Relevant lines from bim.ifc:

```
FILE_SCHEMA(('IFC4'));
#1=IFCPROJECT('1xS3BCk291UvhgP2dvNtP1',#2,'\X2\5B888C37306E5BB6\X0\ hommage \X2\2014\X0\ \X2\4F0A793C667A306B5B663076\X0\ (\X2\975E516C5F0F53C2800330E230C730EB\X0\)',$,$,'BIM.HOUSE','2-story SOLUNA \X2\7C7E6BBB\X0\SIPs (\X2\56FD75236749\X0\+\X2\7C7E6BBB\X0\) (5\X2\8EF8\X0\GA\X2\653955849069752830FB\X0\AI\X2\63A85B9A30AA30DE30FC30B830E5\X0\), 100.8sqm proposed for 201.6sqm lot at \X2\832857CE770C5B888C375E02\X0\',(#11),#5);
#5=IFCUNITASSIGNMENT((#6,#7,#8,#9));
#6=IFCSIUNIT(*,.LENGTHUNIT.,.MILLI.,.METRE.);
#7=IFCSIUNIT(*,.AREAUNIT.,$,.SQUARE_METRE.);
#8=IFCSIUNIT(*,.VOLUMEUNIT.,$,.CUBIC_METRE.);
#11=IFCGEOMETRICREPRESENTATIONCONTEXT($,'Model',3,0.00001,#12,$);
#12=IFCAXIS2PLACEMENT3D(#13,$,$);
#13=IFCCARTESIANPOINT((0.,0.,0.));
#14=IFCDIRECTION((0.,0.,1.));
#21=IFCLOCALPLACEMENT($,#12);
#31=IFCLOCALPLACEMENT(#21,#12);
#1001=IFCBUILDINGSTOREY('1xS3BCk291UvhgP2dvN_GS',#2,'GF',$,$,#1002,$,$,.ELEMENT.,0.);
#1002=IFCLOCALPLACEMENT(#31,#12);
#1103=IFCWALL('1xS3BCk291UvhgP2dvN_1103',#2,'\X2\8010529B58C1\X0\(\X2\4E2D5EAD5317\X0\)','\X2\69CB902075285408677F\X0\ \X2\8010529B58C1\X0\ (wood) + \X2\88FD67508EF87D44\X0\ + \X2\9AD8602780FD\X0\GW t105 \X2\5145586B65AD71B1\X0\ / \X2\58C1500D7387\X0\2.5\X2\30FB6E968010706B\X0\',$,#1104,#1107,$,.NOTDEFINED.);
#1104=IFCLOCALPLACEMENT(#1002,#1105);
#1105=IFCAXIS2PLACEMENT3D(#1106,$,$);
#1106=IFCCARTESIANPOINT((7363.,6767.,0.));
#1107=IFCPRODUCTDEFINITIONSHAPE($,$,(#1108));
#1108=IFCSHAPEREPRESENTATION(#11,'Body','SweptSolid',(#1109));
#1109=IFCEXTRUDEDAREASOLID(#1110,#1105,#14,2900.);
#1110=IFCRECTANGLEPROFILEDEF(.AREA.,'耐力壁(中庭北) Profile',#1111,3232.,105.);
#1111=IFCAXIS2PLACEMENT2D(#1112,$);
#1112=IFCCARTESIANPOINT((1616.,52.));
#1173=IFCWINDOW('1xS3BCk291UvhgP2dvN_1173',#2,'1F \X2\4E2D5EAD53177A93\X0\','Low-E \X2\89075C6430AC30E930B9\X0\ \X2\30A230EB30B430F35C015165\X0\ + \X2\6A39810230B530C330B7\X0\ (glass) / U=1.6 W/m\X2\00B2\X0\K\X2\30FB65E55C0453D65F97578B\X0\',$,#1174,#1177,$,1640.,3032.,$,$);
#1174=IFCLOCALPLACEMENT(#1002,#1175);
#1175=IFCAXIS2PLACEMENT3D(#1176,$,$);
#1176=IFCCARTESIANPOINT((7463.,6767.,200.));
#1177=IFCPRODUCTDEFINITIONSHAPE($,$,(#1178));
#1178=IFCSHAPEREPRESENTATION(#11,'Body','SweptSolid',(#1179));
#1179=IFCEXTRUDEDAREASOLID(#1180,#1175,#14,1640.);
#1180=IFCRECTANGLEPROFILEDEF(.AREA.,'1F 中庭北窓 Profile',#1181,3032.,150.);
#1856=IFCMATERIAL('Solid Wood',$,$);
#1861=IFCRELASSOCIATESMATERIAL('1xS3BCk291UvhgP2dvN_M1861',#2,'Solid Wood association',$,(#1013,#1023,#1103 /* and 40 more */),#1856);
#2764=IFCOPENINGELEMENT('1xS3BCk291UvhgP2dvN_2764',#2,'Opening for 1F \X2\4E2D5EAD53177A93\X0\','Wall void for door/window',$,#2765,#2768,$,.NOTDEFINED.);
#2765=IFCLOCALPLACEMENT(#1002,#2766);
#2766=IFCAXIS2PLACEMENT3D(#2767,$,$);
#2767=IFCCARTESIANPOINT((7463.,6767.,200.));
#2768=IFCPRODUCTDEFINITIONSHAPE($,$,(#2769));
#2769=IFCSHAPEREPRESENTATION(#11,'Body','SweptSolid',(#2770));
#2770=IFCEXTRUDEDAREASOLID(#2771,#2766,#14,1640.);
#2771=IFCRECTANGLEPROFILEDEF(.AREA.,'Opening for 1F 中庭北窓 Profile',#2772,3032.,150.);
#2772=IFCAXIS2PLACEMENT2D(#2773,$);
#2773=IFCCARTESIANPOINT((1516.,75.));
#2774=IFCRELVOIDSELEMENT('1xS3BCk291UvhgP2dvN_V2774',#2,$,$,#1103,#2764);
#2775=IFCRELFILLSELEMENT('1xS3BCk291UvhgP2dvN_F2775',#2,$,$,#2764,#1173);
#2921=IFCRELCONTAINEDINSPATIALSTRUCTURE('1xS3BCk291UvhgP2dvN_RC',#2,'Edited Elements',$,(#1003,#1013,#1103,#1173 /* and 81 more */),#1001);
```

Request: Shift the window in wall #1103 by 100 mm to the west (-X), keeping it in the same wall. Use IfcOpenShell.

```python
import ifcopenshell
import ifcopenshell.api.geometry
import ifcopenshell.util.placement

model = ifcopenshell.open("bim.ifc")

window = model.by_guid("1xS3BCk291UvhgP2dvN_1173")
opening = window.FillsVoids[0].RelatingOpeningElement
wall = opening.VoidsElements[0].RelatingBuildingElement

wall_matrix = ifcopenshell.util.placement.get_local_placement(wall.ObjectPlacement)
shift = wall_matrix[:3, 0] * -100.0
before = ifcopenshell.util.placement.get_local_placement(window.ObjectPlacement)[:3, 3].copy()

# The window is not placed relative to its opening, so move both.
for product in (opening, window):
    matrix = ifcopenshell.util.placement.get_local_placement(product.ObjectPlacement)
    matrix[:3, 3] += shift
    ifcopenshell.api.geometry.edit_object_placement(model, product=product, matrix=matrix, is_si=False)

after = ifcopenshell.util.placement.get_local_placement(window.ObjectPlacement)[:3, 3]
print("window moved by", (after - before).round(3) + 0.0)

model.write("bim-out.ifc")
```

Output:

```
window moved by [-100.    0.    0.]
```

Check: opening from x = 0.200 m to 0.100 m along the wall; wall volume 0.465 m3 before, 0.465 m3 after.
